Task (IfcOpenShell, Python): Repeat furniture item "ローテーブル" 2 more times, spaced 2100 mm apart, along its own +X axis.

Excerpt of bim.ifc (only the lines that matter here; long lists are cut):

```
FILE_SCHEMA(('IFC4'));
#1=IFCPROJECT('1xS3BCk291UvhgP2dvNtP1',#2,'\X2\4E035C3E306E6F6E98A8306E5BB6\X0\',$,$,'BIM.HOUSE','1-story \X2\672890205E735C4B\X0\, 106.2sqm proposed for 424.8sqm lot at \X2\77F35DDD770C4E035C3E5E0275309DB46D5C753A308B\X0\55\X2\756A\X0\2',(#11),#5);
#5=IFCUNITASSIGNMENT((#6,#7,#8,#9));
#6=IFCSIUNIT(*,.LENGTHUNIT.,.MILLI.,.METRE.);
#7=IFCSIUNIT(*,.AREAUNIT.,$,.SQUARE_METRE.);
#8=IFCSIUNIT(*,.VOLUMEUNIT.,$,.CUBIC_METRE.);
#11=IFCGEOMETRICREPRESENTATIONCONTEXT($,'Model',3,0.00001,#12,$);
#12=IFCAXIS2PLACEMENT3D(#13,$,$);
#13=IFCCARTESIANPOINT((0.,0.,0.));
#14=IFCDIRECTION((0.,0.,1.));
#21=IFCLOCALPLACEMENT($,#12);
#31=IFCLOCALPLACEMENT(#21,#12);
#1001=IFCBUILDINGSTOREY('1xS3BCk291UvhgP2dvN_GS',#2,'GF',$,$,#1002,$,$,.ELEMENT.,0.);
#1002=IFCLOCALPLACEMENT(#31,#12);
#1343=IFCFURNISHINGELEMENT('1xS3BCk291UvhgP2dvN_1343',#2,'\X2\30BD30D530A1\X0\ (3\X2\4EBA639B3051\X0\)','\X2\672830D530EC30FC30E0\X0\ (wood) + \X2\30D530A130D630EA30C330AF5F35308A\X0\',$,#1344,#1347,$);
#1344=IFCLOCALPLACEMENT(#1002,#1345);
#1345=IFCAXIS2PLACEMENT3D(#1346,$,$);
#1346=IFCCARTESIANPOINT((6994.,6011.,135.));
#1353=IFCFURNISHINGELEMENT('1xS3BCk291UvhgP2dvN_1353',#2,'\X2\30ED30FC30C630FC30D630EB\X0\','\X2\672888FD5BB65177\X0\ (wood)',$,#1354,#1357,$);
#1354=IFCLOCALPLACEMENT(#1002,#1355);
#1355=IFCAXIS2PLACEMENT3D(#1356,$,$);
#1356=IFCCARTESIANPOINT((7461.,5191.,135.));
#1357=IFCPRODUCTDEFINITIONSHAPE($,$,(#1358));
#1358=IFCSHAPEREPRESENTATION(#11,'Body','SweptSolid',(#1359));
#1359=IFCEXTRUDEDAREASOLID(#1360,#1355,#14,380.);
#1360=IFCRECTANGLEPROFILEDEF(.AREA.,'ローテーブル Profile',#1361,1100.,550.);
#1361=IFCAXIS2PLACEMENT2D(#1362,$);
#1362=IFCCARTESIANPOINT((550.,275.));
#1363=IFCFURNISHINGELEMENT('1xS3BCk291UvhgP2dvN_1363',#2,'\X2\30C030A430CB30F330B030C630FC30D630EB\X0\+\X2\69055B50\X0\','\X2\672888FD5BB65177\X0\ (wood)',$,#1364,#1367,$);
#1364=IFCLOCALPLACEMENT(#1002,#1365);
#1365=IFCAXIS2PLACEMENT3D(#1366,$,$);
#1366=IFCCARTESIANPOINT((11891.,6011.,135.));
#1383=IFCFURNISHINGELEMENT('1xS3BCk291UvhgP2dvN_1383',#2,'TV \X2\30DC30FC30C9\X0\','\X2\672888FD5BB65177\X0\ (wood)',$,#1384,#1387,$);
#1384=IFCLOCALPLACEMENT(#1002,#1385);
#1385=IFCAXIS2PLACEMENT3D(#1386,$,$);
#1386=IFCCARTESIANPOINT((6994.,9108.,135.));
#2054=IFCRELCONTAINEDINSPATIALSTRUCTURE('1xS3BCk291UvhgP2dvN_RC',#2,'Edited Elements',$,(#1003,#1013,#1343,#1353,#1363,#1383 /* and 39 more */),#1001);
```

```python
import ifcopenshell
import ifcopenshell.api.geometry
import ifcopenshell.api.root
import ifcopenshell.util.element
import ifcopenshell.util.placement

model = ifcopenshell.open("bim.ifc")


def reuse_history(source, copy):
    """copy_class also copies each property set's owner history, people and application; keep the originals."""
    for rel in copy.IsDefinedBy:
        if rel.is_a("IfcRelDefinesByProperties") and (history := rel.RelatingPropertyDefinition.OwnerHistory):
            rel.RelatingPropertyDefinition.OwnerHistory = source.OwnerHistory
            ifcopenshell.util.element.remove_deep2(model, history)


source = model.by_guid("1xS3BCk291UvhgP2dvN_1353")
base = ifcopenshell.util.placement.get_local_placement(source.ObjectPlacement)
step = base[:3, 0] * 2100.0

for i in range(1, 3):
    copy = ifcopenshell.api.root.copy_class(model, product=source)
    copy.Representation = ifcopenshell.util.element.copy_deep(
        model, source.Representation, exclude=["IfcGeometricRepresentationContext", "IfcRepresentationMap"]
    )
    reuse_history(source, copy)
    matrix = base.copy()
    matrix[:3, 3] += i * step
    print("added at", matrix[:3, 3].round(3) + 0.0)
    ifcopenshell.api.geometry.edit_object_placement(model, product=copy, matrix=matrix, is_si=False)

model.write("bim_edited.ifc")
```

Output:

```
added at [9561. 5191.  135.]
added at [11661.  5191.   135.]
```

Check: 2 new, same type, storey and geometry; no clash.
